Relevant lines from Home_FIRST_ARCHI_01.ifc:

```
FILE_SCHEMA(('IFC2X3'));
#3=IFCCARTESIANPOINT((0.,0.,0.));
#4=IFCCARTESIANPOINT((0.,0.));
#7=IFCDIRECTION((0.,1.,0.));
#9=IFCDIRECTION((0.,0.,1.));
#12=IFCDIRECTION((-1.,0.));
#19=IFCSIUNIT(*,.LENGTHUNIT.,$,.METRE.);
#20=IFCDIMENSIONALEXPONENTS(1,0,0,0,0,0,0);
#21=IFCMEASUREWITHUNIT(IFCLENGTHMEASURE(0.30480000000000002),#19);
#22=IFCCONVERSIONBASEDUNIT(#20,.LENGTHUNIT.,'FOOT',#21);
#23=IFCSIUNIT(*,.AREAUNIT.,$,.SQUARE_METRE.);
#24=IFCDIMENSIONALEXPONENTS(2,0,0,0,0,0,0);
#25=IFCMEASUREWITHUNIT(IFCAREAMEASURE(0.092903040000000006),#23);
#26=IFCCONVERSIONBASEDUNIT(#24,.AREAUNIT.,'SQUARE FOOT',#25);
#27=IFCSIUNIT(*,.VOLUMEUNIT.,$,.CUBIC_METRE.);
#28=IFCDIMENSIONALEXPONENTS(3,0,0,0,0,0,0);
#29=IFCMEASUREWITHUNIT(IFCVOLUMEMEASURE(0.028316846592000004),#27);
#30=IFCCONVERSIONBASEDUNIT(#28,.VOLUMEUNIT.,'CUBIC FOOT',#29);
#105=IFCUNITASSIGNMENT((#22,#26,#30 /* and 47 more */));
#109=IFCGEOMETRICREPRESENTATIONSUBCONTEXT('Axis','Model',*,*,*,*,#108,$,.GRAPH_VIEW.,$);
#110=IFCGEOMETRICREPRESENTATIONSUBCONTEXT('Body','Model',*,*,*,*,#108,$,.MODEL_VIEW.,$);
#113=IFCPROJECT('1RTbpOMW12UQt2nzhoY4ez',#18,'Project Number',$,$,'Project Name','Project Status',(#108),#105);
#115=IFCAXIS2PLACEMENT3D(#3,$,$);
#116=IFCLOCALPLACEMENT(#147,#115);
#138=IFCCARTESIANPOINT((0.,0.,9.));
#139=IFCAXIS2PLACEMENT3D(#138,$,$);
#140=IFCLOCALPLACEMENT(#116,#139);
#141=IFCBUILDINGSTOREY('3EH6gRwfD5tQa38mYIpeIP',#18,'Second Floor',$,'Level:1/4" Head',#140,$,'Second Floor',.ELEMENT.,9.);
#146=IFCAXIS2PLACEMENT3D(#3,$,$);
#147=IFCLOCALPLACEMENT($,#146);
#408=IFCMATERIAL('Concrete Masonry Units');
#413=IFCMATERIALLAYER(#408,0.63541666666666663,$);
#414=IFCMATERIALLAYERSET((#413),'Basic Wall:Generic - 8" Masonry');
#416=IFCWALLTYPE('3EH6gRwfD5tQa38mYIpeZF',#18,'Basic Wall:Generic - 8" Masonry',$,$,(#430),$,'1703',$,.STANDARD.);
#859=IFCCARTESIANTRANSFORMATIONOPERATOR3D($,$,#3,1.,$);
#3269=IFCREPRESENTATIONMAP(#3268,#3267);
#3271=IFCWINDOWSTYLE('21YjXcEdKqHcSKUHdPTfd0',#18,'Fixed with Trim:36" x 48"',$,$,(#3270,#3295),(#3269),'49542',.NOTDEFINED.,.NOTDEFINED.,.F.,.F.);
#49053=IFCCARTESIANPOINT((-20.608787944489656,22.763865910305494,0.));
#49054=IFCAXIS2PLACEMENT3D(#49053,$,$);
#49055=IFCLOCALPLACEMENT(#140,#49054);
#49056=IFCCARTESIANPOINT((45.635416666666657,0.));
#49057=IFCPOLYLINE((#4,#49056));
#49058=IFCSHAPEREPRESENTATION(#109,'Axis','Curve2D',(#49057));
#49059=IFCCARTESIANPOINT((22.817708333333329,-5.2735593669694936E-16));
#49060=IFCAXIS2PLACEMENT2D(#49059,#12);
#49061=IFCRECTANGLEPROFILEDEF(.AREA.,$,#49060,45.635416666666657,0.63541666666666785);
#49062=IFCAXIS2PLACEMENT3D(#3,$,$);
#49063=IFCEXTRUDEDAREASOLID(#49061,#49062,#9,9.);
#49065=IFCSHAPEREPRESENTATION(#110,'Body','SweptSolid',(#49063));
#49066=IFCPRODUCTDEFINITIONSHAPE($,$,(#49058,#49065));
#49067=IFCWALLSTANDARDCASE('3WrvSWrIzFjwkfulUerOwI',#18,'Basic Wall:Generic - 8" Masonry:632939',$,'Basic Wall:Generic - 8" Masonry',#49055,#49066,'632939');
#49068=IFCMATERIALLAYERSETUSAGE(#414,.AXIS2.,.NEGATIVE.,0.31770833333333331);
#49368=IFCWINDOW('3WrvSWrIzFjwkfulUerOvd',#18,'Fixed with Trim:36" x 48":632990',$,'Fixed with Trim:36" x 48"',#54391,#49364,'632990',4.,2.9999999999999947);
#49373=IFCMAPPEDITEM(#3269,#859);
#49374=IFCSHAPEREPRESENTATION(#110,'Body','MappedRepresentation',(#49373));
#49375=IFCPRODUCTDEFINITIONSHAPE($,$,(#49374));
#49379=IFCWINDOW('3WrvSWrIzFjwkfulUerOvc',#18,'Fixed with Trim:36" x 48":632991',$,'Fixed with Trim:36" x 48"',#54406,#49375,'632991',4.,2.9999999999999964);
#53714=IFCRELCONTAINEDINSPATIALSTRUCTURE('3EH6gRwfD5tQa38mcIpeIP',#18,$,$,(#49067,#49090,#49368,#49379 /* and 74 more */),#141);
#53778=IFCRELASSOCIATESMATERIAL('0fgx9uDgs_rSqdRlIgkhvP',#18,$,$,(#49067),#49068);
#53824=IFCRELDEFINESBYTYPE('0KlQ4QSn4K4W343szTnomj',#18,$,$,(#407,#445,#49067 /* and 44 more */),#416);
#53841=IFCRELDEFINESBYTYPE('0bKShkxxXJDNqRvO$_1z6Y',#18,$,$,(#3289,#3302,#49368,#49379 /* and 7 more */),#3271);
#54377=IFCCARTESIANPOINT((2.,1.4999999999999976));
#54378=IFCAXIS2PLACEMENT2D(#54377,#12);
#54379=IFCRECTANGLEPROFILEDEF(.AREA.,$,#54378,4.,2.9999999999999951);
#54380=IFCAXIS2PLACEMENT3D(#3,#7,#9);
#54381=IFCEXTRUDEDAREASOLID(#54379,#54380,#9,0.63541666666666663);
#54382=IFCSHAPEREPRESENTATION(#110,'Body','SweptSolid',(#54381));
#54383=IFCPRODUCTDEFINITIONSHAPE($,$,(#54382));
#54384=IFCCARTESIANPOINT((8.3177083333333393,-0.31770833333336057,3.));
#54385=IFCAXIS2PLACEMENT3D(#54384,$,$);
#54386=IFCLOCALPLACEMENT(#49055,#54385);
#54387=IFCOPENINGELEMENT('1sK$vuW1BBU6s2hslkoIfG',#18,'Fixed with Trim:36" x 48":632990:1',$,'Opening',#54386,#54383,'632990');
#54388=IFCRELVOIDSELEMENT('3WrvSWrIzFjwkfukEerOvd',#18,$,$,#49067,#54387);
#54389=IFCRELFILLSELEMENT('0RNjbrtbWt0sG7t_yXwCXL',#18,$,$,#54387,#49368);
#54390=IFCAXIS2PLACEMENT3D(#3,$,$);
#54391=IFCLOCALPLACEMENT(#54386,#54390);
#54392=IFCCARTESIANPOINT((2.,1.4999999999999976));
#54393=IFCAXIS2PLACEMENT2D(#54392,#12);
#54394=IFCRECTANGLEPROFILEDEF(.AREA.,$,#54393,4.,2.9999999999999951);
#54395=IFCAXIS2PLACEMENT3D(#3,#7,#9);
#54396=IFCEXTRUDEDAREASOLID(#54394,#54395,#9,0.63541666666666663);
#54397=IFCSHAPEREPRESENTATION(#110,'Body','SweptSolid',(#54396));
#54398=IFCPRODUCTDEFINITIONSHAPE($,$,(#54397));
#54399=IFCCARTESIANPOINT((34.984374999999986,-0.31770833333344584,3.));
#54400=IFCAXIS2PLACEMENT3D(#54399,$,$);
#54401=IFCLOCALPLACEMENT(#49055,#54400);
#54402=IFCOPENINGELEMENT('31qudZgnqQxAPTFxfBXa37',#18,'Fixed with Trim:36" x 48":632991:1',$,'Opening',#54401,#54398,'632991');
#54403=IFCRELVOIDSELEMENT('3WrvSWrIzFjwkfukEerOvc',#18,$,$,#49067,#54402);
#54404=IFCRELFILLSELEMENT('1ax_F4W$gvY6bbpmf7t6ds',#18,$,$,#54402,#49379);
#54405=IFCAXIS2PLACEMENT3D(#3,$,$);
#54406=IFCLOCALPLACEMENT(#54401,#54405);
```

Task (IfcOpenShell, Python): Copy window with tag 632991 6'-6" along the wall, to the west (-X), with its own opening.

```python
import ifcopenshell
import ifcopenshell.api.feature
import ifcopenshell.api.geometry
import ifcopenshell.api.root
import ifcopenshell.geom
import ifcopenshell.util.element
import ifcopenshell.util.placement
import ifcopenshell.util.shape
import ifcopenshell.util.unit

model = ifcopenshell.open("Home_FIRST_ARCHI_01.ifc")
unit_scale = ifcopenshell.util.unit.calculate_unit_scale(model)
settings = ifcopenshell.geom.settings()


def volume(element):
    """Net volume in cubic metres, openings subtracted."""
    shape = ifcopenshell.geom.create_shape(settings, element)
    return ifcopenshell.util.shape.get_volume(shape.geometry)


def reuse_history(source, copy):
    """copy_class also copies each property set's owner history, people and application; keep the originals."""
    for rel in copy.IsDefinedBy:
        if rel.is_a("IfcRelDefinesByProperties") and (history := rel.RelatingPropertyDefinition.OwnerHistory):
            rel.RelatingPropertyDefinition.OwnerHistory = source.OwnerHistory
            ifcopenshell.util.element.remove_deep2(model, history)


window = model.by_guid("3WrvSWrIzFjwkfulUerOvc")
opening = window.FillsVoids[0].RelatingOpeningElement
wall = opening.VoidsElements[0].RelatingBuildingElement
before = volume(wall)
shift = ifcopenshell.util.placement.get_local_placement(wall.ObjectPlacement)[:3, 0] * -78 * 0.0254 / unit_scale

# copy_class copies the void relationship, type, container and properties, but no geometry.
new_opening = ifcopenshell.api.root.copy_class(model, product=opening)
new_opening.Representation = ifcopenshell.util.element.copy_deep(
    model, opening.Representation, exclude=["IfcGeometricRepresentationContext", "IfcRepresentationMap"]
)
new_opening.Name = 'Fixed with Trim:36" x 48"'
new_opening.Tag = None
new_window = ifcopenshell.api.root.copy_class(model, product=window)
new_window.Representation = ifcopenshell.util.element.copy_deep(
    model, window.Representation, exclude=["IfcGeometricRepresentationContext", "IfcRepresentationMap"]
)
new_window.Name = 'Fixed with Trim:36" x 48"'
new_window.Tag = None
reuse_history(window, new_window)
fills = ifcopenshell.api.feature.add_filling(model, opening=new_opening, element=new_window)
fills.OwnerHistory = new_window.OwnerHistory  # required in IFC2X3

for old, new in ((opening, new_opening), (window, new_window)):
    matrix = ifcopenshell.util.placement.get_local_placement(old.ObjectPlacement)
    matrix[:3, 3] += shift
    ifcopenshell.api.geometry.edit_object_placement(model, product=new, matrix=matrix, is_si=False)

after = volume(wall)

print(f"wall volume {before:.3f} -> {after:.3f} m3")

model.write("Home_FIRST_ARCHI_01_v2.ifc")
```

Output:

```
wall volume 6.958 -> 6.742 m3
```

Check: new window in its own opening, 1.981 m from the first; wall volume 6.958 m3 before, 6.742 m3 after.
